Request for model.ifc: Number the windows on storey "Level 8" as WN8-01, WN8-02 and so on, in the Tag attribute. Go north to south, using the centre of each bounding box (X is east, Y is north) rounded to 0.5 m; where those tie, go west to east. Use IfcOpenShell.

First a look at what the model holds.

```python
import ifcopenshell
import ifcopenshell.util.element
import ifcopenshell.util.placement

model = ifcopenshell.open("model.ifc")
print(model.schema)
storey = next(s for s in model.by_type("IfcBuildingStorey") if s.Name == "Level 8")
windows = [e for e in ifcopenshell.util.element.get_decomposition(storey) if e.is_a("IfcWindow")]
for e in sorted(windows, key=lambda e: e.id()):
    origin = ifcopenshell.util.placement.get_local_placement(e.ObjectPlacement)[:3, 3]
    print(e.id(), e.Tag, e.Name, origin.round(2) + 0.0, sep=" | ")
```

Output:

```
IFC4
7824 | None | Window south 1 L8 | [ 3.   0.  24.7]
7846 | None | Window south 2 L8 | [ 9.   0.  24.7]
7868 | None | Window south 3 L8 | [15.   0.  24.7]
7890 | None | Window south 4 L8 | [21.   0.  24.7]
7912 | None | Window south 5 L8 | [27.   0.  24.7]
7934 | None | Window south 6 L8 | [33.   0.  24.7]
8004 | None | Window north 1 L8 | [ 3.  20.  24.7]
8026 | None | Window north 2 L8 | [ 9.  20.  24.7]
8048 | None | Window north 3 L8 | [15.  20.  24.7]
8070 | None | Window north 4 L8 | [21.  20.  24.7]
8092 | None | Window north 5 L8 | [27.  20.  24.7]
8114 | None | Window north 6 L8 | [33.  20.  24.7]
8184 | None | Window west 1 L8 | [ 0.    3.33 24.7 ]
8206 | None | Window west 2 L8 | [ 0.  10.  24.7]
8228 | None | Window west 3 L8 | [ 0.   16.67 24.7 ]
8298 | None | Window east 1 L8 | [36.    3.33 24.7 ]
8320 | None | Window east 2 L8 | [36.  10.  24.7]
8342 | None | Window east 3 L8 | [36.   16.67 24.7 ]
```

```python
import ifcopenshell
import ifcopenshell.geom
import ifcopenshell.util.element
import ifcopenshell.util.shape

model = ifcopenshell.open("model.ifc")
settings = ifcopenshell.geom.settings()
settings.set("use-world-coords", True)


def centre(element):
    shape = ifcopenshell.geom.create_shape(settings, element)
    return ifcopenshell.util.shape.get_bbox_centroid(shape.geometry)


storey = next(s for s in model.by_type("IfcBuildingStorey") if s.Name == "Level 8")
windows = [e for e in ifcopenshell.util.element.get_decomposition(storey) if e.is_a("IfcWindow")]

# Insertion points can sit at a corner or the storey origin, so sort by the geometry (in metres).
centres = {e: centre(e) for e in windows}
windows.sort(key=lambda e: (-round(centres[e][1] / 0.5), centres[e][0]))

for i, e in enumerate(windows, start=1):
    number = f"WN8-{i:02d}"
    e.Tag = number
    print(e.id(), number)

model.write("model_updated.ifc")
```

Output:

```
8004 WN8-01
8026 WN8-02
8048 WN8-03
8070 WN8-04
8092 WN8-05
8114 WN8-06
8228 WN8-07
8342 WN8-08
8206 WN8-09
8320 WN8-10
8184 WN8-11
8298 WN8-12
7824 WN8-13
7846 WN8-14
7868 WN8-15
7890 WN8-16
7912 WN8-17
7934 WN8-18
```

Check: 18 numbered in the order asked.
